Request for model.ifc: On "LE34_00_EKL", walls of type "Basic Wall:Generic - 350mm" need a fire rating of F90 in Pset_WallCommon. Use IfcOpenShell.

First a look at what the model holds.

```python
import ifcopenshell
import ifcopenshell.util.element

model = ifcopenshell.open("model.ifc")
print(model.schema)
storey = next(s for s in model.by_type("IfcBuildingStorey") if s.Name == "LE34_00_EKL")
walls = [e for e in ifcopenshell.util.element.get_decomposition(storey) if e.is_a("IfcWall")]
seen = {}
for e in walls:
    element_type = ifcopenshell.util.element.get_type(e)
    key = (element_type.Name if element_type != e and element_type else None, ifcopenshell.util.element.get_pset(e, "Pset_WallCommon", "FireRating"))
    seen[key] = seen.get(key, 0) + 1
for (name, value), count in sorted(seen.items(), key=str):
    print(count, "x", name, "|", value)
```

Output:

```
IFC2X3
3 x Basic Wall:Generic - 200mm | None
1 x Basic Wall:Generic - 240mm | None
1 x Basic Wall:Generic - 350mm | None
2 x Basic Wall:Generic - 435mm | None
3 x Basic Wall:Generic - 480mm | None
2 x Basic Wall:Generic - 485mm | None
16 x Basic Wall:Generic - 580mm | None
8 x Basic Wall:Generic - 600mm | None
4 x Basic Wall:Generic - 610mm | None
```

```python
import ifcopenshell
import ifcopenshell.api.pset
import ifcopenshell.util.element

model = ifcopenshell.open("model.ifc")

storey = next(s for s in model.by_type("IfcBuildingStorey") if s.Name == "LE34_00_EKL")
walls = [e for e in ifcopenshell.util.element.get_decomposition(storey) if e.is_a("IfcWall")]

count = 0
for e in walls:
    element_type = ifcopenshell.util.element.get_type(e)
    if element_type in (None, e) or element_type.Name != "Basic Wall:Generic - 350mm":
        continue
    # add_pset returns the element's existing set when there is one.
    pset = ifcopenshell.api.pset.add_pset(model, product=e, name="Pset_WallCommon")
    ifcopenshell.api.pset.edit_pset(model, pset=pset, properties={"FireRating": "F90"})
    count += 1

print(count, "walls updated")

model.write("model_rev.ifc")
```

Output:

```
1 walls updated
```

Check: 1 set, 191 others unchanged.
